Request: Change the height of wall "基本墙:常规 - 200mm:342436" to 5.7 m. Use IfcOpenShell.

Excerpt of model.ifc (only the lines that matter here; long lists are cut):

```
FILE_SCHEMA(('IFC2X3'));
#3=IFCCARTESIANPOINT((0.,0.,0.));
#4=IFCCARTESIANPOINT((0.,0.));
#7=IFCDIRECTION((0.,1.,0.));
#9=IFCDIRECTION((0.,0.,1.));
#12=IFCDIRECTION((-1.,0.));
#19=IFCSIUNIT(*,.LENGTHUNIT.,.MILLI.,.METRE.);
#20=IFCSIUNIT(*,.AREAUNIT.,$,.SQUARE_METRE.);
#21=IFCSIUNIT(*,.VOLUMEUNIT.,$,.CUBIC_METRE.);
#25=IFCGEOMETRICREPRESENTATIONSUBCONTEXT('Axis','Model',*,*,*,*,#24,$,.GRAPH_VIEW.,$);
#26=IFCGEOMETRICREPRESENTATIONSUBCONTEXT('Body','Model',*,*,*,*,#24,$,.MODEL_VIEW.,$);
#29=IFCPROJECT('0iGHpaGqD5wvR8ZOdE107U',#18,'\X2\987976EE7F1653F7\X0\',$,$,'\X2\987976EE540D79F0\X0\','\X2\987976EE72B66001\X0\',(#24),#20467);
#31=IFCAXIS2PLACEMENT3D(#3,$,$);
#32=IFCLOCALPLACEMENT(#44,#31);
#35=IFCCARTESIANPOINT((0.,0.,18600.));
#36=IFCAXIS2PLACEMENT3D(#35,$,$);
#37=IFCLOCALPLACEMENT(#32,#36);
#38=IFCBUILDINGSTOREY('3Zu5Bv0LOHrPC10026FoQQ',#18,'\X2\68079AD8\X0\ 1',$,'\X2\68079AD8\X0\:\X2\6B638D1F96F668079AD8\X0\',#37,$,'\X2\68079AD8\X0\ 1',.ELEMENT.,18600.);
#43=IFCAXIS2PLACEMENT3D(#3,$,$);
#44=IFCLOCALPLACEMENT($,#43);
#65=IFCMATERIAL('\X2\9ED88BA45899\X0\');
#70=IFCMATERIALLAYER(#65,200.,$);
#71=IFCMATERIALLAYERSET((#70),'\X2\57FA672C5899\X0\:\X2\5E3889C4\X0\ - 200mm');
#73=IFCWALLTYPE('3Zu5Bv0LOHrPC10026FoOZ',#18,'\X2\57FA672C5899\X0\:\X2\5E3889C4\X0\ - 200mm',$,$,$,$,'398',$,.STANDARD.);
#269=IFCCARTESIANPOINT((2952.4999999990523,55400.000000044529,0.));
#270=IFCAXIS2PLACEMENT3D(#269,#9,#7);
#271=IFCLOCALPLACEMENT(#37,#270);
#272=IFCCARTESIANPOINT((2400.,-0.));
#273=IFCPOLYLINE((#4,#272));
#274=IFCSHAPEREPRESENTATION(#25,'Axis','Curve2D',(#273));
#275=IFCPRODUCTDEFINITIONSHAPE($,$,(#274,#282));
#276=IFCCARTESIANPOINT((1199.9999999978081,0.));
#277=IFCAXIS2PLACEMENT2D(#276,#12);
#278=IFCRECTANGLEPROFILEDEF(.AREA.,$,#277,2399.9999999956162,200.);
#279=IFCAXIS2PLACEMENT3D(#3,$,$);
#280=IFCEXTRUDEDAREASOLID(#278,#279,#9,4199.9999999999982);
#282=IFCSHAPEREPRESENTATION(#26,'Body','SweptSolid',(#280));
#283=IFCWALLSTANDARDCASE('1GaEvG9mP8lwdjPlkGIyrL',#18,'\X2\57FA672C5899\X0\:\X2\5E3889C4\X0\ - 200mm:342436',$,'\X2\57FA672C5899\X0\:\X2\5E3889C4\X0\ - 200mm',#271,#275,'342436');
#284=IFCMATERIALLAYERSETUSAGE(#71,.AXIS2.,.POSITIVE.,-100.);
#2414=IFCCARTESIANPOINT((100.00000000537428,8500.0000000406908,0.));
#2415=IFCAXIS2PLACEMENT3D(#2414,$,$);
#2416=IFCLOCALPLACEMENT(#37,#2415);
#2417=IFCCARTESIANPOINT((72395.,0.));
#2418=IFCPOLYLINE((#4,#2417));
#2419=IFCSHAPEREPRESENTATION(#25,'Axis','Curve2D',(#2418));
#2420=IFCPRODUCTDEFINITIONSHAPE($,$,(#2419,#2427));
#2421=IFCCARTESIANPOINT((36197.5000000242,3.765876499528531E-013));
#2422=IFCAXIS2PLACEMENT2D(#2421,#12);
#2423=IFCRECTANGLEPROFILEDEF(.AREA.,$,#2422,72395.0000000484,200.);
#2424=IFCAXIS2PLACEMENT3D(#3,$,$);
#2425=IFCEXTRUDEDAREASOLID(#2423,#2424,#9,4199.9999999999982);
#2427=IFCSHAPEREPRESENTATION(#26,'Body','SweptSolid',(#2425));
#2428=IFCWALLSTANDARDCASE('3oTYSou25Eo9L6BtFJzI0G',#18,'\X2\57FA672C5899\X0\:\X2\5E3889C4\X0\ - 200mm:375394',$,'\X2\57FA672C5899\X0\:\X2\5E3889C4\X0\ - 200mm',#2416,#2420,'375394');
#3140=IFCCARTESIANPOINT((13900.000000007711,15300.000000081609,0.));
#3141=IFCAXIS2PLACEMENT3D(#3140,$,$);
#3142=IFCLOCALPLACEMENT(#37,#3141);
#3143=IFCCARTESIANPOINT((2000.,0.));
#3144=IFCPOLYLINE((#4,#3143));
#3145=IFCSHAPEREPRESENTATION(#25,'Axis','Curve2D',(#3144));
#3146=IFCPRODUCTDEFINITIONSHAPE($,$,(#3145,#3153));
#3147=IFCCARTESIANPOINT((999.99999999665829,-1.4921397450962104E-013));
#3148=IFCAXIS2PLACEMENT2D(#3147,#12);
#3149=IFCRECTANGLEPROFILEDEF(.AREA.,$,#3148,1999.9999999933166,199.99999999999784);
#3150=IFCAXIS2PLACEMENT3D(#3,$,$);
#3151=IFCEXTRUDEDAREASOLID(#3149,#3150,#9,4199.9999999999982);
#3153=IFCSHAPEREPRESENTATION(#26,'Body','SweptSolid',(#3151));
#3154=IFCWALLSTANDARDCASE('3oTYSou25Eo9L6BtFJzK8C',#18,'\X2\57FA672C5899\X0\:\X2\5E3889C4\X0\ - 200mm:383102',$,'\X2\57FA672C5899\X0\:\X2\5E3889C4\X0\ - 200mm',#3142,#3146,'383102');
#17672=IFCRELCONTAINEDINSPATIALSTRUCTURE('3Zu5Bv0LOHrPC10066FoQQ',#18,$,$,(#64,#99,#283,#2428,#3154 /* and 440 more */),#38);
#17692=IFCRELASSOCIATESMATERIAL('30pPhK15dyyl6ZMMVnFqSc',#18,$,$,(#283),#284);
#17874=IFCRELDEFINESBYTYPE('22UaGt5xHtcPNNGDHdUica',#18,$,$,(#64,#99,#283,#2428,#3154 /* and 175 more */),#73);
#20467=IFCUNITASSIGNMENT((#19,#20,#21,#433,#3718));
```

```python
import ifcopenshell
import ifcopenshell.geom
import ifcopenshell.util.representation
import ifcopenshell.util.shape
import ifcopenshell.util.unit

model = ifcopenshell.open("model.ifc")
unit_scale = ifcopenshell.util.unit.calculate_unit_scale(model)
settings = ifcopenshell.geom.settings()


def volume(element):
    """Net volume in cubic metres, openings subtracted."""
    shape = ifcopenshell.geom.create_shape(settings, element)
    return ifcopenshell.util.shape.get_volume(shape.geometry)


wall = model.by_id(283)
before = volume(wall)

body = ifcopenshell.util.representation.get_representation(wall, "Model", "Body")
solid = body.Items[0]
old_height = solid.Depth
solid.Depth = 5.7 / unit_scale
after = volume(wall)

print(f"height {old_height:g} -> {solid.Depth:g}, volume {before:.3f} -> {after:.3f} m3")

model.write("model_rev.ifc")
```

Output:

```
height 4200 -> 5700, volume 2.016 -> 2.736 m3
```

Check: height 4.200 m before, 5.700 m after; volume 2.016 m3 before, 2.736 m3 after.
